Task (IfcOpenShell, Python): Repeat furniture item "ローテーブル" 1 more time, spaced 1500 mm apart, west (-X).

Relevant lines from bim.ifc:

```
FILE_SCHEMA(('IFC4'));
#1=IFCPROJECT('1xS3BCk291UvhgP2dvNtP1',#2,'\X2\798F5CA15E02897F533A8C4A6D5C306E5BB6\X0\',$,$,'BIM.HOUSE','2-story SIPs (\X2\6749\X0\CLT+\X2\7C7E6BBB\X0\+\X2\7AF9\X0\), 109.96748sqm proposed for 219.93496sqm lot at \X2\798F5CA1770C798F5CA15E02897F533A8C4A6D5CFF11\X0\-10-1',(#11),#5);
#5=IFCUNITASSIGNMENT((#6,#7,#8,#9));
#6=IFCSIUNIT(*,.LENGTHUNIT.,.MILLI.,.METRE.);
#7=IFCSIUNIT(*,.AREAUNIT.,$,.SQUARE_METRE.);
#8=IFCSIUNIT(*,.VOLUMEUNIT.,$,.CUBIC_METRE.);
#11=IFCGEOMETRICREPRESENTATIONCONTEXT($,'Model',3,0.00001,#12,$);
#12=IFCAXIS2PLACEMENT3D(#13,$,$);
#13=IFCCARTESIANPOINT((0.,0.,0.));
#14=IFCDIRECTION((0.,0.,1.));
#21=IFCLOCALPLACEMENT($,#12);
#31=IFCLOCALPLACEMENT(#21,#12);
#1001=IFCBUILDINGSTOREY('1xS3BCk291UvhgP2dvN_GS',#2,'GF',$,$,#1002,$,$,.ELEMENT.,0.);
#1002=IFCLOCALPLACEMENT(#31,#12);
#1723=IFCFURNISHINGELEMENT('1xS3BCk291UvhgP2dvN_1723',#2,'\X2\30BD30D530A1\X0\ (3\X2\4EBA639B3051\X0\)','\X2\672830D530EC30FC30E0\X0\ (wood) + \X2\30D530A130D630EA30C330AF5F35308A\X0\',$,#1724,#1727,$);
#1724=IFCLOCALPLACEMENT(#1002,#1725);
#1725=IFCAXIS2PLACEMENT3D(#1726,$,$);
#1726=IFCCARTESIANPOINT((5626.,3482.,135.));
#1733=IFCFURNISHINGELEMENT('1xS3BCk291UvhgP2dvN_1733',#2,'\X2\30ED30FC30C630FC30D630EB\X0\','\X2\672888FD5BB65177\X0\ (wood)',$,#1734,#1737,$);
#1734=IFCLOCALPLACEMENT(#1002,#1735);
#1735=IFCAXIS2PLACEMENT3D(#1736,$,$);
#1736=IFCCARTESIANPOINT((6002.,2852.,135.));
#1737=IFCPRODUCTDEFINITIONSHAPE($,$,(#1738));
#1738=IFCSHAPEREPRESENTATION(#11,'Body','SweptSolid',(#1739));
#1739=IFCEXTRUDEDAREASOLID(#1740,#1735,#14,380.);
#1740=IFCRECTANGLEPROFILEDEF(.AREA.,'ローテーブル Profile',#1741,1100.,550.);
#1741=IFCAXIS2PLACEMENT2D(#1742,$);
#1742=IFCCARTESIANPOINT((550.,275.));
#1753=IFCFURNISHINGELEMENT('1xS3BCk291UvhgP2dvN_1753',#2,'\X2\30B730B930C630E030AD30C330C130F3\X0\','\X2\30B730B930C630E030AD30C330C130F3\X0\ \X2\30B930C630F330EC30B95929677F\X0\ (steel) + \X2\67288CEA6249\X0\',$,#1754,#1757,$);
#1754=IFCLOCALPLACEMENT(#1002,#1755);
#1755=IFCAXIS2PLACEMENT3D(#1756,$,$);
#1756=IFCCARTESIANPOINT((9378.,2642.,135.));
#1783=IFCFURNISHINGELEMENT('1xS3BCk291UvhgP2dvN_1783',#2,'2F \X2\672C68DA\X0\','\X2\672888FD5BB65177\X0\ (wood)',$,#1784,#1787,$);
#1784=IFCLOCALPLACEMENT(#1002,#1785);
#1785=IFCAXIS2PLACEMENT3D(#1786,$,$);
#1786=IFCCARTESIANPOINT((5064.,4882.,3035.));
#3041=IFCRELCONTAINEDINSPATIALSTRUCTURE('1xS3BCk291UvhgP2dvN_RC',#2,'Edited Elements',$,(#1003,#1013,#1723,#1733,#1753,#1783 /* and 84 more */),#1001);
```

```python
import numpy as np
import ifcopenshell
import ifcopenshell.api.geometry
import ifcopenshell.api.root
import ifcopenshell.util.element
import ifcopenshell.util.placement

model = ifcopenshell.open("bim.ifc")


def reuse_history(source, copy):
    """copy_class also copies each property set's owner history, people and application; keep the originals."""
    for rel in copy.IsDefinedBy:
        if rel.is_a("IfcRelDefinesByProperties") and (history := rel.RelatingPropertyDefinition.OwnerHistory):
            rel.RelatingPropertyDefinition.OwnerHistory = source.OwnerHistory
            ifcopenshell.util.element.remove_deep2(model, history)


source = model.by_guid("1xS3BCk291UvhgP2dvN_1733")
base = ifcopenshell.util.placement.get_local_placement(source.ObjectPlacement)
step = np.array([-1.0, 0.0, 0.0]) * 1500.0

for i in range(1, 2):
    copy = ifcopenshell.api.root.copy_class(model, product=source)
    copy.Representation = ifcopenshell.util.element.copy_deep(
        model, source.Representation, exclude=["IfcGeometricRepresentationContext", "IfcRepresentationMap"]
    )
    reuse_history(source, copy)
    matrix = base.copy()
    matrix[:3, 3] += i * step
    print("added at", matrix[:3, 3].round(3) + 0.0)
    ifcopenshell.api.geometry.edit_object_placement(model, product=copy, matrix=matrix, is_si=False)

model.write("bim-out.ifc")
```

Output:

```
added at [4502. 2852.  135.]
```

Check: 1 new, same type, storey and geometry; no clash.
